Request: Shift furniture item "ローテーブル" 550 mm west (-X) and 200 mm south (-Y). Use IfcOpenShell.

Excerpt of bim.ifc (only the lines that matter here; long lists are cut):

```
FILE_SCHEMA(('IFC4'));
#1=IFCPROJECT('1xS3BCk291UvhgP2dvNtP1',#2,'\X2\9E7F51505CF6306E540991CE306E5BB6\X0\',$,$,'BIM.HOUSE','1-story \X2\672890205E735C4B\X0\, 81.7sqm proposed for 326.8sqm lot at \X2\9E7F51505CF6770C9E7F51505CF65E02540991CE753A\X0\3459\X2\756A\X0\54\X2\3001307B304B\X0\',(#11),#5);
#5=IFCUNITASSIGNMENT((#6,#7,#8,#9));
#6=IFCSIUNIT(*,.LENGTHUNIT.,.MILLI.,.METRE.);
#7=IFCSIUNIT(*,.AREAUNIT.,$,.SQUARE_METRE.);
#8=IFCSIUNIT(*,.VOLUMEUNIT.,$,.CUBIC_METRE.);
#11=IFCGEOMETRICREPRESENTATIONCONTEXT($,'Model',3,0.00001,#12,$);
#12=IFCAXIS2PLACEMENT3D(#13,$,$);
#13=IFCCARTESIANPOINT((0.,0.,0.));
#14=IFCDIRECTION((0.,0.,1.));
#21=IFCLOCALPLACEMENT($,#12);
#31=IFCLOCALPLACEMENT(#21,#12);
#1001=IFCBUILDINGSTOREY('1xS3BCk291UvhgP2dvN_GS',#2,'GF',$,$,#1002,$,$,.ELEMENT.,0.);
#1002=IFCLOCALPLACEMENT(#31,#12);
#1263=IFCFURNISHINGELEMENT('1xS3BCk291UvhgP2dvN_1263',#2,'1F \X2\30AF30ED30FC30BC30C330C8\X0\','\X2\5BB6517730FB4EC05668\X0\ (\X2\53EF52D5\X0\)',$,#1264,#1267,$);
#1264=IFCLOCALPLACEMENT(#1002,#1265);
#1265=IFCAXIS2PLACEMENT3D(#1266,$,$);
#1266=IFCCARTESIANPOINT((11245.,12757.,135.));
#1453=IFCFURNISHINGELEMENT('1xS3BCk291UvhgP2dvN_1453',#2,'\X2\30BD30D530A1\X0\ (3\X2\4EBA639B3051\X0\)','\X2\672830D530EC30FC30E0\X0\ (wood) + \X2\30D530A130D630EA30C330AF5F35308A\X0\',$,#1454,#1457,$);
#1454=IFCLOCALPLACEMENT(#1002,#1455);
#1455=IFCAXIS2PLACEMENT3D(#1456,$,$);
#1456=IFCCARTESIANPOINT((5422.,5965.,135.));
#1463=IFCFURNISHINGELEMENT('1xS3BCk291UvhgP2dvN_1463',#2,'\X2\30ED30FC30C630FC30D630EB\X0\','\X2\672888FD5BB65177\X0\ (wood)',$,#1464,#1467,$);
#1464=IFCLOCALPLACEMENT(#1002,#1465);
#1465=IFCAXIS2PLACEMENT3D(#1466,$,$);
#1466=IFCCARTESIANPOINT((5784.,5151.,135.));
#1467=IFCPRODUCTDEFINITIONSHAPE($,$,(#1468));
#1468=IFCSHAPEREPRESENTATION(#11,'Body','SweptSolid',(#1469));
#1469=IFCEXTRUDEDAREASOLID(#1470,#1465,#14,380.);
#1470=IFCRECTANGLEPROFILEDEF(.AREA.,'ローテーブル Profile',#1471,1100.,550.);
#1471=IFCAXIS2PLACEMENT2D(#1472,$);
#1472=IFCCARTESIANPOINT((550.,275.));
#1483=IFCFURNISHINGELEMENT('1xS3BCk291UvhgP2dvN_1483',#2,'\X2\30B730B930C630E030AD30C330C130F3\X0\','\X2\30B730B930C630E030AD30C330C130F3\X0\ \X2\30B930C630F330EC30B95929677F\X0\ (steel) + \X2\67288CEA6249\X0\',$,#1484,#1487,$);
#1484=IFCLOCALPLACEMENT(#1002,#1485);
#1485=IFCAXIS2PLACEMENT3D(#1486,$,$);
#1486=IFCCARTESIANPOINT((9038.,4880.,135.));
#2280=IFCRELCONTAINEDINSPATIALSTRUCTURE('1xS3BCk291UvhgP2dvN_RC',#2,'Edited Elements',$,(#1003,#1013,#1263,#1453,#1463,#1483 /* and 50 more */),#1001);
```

```python
import ifcopenshell
import ifcopenshell.api.geometry
import ifcopenshell.util.placement
import ifcopenshell.util.unit

model = ifcopenshell.open("bim.ifc")
unit_scale = ifcopenshell.util.unit.calculate_unit_scale(model)

item = model.by_guid("1xS3BCk291UvhgP2dvN_1463")
matrix = ifcopenshell.util.placement.get_local_placement(item.ObjectPlacement)
matrix[0, 3] -= 0.55 / unit_scale
matrix[1, 3] -= 0.2 / unit_scale
ifcopenshell.api.geometry.edit_object_placement(model, product=item, matrix=matrix, is_si=False)

print(ifcopenshell.util.placement.get_local_placement(item.ObjectPlacement).round(3) + 0.0)

model.write("bim_edited.ifc")
```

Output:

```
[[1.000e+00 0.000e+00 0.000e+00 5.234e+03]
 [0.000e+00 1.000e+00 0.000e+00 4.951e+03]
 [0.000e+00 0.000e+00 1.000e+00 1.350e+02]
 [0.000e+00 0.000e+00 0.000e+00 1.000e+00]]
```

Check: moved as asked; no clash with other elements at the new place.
